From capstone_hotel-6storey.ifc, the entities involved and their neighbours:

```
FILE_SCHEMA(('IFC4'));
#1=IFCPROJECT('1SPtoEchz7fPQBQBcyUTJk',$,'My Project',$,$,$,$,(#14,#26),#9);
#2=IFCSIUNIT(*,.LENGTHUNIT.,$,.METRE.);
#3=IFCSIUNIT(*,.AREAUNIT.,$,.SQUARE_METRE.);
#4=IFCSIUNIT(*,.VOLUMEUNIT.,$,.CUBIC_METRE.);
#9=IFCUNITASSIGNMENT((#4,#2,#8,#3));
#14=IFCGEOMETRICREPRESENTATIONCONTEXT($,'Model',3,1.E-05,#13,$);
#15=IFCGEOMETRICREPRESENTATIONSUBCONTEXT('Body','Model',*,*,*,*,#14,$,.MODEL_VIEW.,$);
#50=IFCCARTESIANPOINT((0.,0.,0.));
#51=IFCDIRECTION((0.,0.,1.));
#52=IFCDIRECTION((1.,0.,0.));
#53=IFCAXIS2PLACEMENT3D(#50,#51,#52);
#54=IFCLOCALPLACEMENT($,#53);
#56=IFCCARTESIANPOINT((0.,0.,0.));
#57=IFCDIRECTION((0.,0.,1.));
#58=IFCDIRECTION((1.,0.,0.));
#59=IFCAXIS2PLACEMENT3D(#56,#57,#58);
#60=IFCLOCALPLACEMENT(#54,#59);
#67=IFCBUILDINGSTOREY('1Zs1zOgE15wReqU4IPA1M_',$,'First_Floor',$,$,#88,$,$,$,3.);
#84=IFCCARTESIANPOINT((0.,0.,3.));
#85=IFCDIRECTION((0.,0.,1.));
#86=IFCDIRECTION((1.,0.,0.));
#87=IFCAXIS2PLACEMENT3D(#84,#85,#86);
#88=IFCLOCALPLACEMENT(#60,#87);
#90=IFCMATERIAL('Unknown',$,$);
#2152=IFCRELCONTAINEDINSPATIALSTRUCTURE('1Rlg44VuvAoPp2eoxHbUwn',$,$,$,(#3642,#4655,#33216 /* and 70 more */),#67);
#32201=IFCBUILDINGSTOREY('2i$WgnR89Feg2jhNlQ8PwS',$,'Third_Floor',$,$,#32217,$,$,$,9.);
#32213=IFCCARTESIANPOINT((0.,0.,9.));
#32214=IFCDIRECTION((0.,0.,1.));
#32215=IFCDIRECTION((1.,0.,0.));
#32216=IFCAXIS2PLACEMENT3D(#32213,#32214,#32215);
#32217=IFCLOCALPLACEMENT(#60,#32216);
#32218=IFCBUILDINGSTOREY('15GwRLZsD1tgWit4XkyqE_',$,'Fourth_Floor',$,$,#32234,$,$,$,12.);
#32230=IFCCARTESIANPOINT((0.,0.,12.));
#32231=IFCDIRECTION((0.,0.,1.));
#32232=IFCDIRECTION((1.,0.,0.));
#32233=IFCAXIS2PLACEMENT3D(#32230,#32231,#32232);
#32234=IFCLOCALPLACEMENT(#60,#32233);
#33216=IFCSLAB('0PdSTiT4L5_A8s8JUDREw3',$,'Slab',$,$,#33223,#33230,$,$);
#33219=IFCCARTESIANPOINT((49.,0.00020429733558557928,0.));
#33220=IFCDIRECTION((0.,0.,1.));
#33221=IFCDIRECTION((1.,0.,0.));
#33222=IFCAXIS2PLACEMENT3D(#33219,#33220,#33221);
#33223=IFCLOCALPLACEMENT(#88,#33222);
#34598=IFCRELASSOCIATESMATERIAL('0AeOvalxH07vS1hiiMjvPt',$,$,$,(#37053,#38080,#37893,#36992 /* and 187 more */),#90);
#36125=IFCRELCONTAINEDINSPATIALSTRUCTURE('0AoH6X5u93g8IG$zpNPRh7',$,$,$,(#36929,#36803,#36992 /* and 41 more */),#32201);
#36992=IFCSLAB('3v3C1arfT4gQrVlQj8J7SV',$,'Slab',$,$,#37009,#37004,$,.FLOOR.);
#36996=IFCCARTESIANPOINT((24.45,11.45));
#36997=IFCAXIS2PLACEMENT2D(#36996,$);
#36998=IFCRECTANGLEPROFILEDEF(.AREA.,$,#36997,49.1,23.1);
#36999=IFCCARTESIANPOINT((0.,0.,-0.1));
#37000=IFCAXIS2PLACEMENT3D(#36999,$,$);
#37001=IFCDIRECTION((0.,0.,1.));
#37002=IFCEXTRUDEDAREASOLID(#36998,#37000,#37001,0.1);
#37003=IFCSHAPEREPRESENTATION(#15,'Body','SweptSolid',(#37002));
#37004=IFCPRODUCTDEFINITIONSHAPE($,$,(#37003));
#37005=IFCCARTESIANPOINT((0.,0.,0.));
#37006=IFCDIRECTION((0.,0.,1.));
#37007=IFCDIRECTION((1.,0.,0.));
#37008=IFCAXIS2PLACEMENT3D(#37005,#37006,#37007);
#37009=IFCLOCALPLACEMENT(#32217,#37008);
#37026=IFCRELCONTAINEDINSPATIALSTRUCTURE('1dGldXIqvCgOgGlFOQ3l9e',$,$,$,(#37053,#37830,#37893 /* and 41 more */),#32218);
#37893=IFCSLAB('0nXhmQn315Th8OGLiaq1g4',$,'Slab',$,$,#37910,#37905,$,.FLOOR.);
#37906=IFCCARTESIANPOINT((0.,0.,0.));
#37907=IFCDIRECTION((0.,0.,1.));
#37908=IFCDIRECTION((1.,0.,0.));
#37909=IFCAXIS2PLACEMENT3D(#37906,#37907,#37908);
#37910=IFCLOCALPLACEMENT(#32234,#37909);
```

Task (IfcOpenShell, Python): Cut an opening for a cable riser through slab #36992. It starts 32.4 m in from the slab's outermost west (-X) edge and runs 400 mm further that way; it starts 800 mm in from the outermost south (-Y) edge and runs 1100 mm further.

```python
import numpy as np
import ifcopenshell
import ifcopenshell.api.feature
import ifcopenshell.api.geometry
import ifcopenshell.api.root
import ifcopenshell.geom
import ifcopenshell.util.placement
import ifcopenshell.util.representation
import ifcopenshell.util.shape
import ifcopenshell.util.unit

model = ifcopenshell.open("capstone_hotel-6storey.ifc")
unit_scale = ifcopenshell.util.unit.calculate_unit_scale(model)
settings = ifcopenshell.geom.settings()


def volume(element):
    """Net volume in cubic metres, openings subtracted."""
    shape = ifcopenshell.geom.create_shape(settings, element)
    return ifcopenshell.util.shape.get_volume(shape.geometry)


slab = model.by_guid("3v3C1arfT4gQrVlQj8J7SV")
before = volume(slab)

# Extent in the slab's own axes, in metres. The edges named are its -X and -Y sides.
slab_shape = ifcopenshell.geom.create_shape(settings, slab)
vertices = ifcopenshell.util.shape.get_vertices(slab_shape.geometry)
x_min, y_min, bottom = vertices.min(axis=0)
top = vertices[:, 2].max()

opening = ifcopenshell.api.root.create_entity(model, ifc_class="IfcOpeningElement", name="Cable riser opening", predefined_type="OPENING")
context = ifcopenshell.util.representation.get_context(model, "Model", "Body", "MODEL_VIEW")
width, depth = 0.4, 1.1
outline = [(0.0, 0.0), (width, 0.0), (width, depth), (0.0, depth), (0.0, 0.0)]
# Overshoot both faces by 50 mm so the cut is clean.
shape = ifcopenshell.api.geometry.add_slab_representation(
    model, context=context, depth=top - bottom + 0.1, polyline=outline
)
ifcopenshell.api.geometry.assign_representation(model, product=opening, representation=shape)

matrix = ifcopenshell.util.placement.get_local_placement(slab.ObjectPlacement)
matrix[:, 3] = matrix @ np.append(np.array([x_min + 32.4, y_min + 0.8, bottom - 0.05]) / unit_scale, 1.0)
ifcopenshell.api.geometry.edit_object_placement(model, product=opening, matrix=matrix, is_si=False)
ifcopenshell.api.feature.add_feature(model, feature=opening, element=slab)

after = volume(slab)

print(f"slab volume {before:.3f} -> {after:.3f} m3")

model.write("capstone_hotel-6storey-out.ifc")
```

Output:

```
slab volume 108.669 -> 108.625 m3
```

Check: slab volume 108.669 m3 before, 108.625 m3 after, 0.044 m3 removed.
